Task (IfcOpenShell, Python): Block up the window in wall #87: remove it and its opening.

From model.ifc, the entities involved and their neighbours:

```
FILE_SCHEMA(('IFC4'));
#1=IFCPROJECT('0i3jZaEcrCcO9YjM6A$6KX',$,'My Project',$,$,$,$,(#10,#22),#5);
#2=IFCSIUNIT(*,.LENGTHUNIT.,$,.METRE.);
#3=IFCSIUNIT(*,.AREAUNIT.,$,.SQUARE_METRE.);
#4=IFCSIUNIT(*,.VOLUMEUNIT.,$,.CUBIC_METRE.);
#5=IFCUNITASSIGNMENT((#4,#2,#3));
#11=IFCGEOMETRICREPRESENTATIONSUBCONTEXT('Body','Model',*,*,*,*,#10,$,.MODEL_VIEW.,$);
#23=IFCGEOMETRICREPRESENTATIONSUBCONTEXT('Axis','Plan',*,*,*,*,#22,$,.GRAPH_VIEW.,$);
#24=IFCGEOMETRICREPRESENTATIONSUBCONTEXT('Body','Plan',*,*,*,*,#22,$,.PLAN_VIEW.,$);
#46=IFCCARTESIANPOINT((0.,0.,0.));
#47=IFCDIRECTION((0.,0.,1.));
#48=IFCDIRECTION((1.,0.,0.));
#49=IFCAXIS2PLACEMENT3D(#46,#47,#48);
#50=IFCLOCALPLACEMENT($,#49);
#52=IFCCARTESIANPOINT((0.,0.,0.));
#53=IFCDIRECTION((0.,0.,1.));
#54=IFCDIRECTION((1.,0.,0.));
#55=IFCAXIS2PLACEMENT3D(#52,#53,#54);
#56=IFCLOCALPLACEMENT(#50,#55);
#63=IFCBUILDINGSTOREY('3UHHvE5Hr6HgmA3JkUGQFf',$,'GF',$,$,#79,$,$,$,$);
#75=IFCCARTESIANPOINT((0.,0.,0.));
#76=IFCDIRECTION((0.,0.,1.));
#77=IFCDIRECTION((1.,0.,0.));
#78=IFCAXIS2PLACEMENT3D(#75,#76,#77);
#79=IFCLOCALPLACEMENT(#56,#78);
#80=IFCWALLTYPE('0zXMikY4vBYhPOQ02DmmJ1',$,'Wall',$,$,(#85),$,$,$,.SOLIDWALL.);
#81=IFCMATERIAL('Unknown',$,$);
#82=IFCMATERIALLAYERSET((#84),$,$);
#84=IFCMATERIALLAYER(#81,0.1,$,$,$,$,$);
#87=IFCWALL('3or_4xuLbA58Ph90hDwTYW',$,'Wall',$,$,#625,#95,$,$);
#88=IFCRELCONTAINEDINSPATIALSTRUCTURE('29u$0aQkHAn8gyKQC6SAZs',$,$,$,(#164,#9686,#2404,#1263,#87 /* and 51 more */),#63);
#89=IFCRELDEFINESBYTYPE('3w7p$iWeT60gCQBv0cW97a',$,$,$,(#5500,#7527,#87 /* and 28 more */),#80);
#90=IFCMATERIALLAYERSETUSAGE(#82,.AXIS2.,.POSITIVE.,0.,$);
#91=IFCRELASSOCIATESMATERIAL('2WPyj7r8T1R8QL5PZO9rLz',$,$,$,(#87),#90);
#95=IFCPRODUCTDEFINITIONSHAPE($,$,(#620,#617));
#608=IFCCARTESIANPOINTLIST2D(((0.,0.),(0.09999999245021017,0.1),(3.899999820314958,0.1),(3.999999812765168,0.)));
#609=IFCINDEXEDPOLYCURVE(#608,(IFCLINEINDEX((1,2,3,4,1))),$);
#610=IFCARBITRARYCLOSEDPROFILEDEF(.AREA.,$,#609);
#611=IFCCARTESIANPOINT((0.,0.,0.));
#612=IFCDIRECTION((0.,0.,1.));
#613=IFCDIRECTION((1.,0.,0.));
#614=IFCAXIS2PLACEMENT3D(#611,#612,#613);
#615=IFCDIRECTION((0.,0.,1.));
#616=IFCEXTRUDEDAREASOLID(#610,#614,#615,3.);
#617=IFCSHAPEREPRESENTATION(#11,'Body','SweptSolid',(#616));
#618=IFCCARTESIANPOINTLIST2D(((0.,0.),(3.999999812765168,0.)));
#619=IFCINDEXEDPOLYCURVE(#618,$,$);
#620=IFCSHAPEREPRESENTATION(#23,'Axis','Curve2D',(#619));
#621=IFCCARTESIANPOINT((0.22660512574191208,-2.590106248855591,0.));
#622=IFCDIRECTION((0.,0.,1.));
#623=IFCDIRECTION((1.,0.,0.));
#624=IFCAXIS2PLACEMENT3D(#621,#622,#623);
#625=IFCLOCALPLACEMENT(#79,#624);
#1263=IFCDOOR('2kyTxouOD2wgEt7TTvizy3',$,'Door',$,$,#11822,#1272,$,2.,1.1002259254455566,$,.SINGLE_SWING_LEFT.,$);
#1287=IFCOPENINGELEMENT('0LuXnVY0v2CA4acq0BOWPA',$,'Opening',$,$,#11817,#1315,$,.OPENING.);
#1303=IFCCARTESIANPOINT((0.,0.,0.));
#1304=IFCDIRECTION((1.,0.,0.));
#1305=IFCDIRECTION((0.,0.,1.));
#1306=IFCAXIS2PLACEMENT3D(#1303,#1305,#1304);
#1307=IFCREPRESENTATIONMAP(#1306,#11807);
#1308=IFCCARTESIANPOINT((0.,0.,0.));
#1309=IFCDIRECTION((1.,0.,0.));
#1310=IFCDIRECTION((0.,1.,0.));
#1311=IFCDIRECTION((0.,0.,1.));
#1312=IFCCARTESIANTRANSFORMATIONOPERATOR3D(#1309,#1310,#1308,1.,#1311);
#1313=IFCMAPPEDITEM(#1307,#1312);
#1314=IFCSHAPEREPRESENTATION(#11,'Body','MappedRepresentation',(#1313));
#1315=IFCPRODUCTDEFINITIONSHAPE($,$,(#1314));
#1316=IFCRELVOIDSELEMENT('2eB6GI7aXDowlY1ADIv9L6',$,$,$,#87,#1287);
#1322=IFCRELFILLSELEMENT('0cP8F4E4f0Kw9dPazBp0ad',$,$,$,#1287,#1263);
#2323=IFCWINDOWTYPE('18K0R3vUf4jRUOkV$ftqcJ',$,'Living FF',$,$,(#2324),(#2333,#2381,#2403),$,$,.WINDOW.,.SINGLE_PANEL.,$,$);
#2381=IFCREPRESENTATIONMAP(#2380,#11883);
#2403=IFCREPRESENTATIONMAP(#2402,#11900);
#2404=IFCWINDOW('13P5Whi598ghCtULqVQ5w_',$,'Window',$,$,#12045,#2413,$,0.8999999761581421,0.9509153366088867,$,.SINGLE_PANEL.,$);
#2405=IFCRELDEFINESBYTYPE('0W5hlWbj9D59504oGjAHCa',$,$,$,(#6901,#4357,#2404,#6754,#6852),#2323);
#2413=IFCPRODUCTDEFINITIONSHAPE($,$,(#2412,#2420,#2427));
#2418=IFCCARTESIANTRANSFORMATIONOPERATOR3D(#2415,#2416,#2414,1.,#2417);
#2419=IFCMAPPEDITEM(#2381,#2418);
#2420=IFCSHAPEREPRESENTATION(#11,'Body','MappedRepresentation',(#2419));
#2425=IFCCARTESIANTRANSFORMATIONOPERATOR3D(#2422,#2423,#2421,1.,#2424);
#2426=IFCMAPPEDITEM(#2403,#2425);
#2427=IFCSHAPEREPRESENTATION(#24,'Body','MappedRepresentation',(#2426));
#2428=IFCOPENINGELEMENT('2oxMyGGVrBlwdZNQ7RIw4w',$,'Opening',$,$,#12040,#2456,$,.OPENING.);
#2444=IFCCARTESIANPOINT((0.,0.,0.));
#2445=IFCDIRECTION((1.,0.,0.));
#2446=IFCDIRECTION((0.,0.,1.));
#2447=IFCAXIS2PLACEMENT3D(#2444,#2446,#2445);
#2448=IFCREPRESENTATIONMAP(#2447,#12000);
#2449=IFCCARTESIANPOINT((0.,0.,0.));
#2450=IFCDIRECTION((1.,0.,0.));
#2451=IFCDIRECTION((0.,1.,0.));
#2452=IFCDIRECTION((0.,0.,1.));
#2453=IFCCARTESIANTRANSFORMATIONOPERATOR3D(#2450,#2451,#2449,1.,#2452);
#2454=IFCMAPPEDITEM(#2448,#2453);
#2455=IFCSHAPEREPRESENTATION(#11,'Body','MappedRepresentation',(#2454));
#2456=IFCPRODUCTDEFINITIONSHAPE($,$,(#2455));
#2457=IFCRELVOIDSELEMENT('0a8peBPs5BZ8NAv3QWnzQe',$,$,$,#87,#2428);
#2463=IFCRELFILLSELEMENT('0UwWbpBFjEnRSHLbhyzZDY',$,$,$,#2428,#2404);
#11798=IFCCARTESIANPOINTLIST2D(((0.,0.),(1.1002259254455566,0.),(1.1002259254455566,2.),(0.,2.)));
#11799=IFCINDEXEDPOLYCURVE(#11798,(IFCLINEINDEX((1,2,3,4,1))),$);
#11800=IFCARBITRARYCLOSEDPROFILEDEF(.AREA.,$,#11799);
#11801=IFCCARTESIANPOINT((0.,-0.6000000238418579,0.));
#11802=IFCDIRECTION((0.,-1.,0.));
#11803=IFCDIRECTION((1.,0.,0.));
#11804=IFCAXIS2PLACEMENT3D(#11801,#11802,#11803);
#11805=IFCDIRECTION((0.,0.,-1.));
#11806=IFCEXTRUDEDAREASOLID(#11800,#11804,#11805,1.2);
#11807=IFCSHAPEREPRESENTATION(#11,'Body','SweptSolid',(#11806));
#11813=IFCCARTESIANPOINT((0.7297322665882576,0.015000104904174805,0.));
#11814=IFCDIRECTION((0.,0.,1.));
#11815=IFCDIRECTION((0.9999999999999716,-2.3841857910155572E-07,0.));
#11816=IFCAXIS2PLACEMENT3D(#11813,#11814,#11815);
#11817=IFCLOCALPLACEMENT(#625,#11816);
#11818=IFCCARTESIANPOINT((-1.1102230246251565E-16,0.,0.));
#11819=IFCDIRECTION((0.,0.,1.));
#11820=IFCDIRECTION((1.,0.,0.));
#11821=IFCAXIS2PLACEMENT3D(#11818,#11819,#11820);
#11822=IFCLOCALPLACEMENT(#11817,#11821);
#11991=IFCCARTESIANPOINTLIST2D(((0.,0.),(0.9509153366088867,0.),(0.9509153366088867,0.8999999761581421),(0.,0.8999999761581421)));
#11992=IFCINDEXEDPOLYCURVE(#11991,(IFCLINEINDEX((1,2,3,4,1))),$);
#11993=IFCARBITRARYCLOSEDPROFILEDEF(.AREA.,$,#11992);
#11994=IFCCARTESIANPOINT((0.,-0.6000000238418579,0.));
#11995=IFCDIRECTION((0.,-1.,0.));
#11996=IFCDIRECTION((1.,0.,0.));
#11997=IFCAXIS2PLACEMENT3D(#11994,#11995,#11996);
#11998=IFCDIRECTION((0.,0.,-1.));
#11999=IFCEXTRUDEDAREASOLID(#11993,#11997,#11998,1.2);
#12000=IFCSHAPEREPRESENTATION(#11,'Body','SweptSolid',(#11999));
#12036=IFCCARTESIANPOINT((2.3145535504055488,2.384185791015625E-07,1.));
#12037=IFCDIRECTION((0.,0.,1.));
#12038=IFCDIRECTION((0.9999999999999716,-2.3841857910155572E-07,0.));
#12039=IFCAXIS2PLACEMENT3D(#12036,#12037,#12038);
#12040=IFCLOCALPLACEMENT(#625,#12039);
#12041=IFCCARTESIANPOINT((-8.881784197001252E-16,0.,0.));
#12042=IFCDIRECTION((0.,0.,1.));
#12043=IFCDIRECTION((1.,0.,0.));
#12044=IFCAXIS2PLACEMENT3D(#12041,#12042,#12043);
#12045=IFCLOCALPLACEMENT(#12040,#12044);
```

```python
import ifcopenshell
import ifcopenshell.api.feature
import ifcopenshell.api.root
import ifcopenshell.geom
import ifcopenshell.util.shape

model = ifcopenshell.open("model.ifc")
settings = ifcopenshell.geom.settings()


def volume(element):
    """Net volume in cubic metres, openings subtracted."""
    shape = ifcopenshell.geom.create_shape(settings, element)
    return ifcopenshell.util.shape.get_volume(shape.geometry)


window = model.by_guid("13P5Whi598ghCtULqVQ5w_")
opening = window.FillsVoids[0].RelatingOpeningElement
wall = opening.VoidsElements[0].RelatingBuildingElement
before = volume(wall)

ifcopenshell.api.root.remove_product(model, product=window)
ifcopenshell.api.feature.remove_feature(model, feature=opening)

after = volume(wall)

print(f"wall volume {before:.3f} -> {after:.3f} m3")

model.write("model-out.ifc")
```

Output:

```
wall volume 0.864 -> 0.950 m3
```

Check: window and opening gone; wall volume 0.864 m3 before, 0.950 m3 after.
